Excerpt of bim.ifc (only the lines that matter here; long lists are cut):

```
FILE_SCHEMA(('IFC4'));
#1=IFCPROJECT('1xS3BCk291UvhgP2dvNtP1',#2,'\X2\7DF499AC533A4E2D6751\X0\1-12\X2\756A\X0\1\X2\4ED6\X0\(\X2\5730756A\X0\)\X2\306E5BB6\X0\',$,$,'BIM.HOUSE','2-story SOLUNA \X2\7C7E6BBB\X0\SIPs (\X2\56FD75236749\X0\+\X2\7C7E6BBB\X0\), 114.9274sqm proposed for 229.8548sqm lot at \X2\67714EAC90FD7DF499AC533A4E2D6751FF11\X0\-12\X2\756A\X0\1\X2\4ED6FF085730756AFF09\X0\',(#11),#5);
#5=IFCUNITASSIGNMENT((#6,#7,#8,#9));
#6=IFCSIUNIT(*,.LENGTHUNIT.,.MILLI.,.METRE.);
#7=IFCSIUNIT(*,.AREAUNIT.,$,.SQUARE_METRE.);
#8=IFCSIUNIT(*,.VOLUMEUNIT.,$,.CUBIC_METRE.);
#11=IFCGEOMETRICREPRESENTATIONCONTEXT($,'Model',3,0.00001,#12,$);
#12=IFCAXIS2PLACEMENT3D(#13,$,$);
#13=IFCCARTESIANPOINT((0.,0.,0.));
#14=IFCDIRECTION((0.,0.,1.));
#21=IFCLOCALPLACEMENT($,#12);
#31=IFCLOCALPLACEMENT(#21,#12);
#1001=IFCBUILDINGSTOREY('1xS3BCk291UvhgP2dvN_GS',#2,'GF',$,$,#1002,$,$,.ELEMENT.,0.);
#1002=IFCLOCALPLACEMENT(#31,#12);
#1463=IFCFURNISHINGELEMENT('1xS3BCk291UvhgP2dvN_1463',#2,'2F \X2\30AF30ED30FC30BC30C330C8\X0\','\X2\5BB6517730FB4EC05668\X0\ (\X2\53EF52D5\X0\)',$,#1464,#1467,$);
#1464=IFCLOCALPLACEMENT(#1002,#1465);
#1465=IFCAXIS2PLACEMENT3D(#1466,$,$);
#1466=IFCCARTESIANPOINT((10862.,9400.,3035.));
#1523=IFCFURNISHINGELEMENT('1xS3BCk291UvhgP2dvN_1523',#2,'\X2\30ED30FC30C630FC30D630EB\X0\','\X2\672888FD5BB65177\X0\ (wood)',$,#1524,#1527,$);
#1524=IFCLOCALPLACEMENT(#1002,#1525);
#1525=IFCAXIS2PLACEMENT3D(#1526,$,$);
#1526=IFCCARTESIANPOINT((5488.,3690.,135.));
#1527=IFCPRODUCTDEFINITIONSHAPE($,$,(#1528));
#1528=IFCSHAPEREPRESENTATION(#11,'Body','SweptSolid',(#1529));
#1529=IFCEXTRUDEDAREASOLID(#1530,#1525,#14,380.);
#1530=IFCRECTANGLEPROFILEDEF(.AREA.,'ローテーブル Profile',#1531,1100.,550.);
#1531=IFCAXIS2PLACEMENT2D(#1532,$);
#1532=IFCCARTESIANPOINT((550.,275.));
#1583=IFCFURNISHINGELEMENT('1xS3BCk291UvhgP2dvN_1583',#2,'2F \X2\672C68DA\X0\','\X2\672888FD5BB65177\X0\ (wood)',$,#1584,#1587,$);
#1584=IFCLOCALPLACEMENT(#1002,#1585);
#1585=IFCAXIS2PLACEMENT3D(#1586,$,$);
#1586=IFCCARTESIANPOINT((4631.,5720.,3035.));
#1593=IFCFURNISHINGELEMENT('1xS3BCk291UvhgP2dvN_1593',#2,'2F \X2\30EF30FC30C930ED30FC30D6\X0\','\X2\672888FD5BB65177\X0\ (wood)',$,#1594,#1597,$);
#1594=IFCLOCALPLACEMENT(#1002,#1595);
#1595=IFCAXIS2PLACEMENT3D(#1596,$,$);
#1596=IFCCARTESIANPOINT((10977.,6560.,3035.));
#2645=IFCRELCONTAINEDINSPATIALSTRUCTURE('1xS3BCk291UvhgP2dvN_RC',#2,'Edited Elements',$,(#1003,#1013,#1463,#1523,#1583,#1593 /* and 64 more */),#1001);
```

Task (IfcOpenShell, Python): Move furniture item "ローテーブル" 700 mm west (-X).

```python
import ifcopenshell
import ifcopenshell.api.geometry
import ifcopenshell.util.placement

model = ifcopenshell.open("bim.ifc")

item = model.by_guid("1xS3BCk291UvhgP2dvN_1523")
matrix = ifcopenshell.util.placement.get_local_placement(item.ObjectPlacement)
matrix[0, 3] -= 700.0
ifcopenshell.api.geometry.edit_object_placement(model, product=item, matrix=matrix, is_si=False)

print(ifcopenshell.util.placement.get_local_placement(item.ObjectPlacement).round(3) + 0.0)

model.write("bim_updated.ifc")
```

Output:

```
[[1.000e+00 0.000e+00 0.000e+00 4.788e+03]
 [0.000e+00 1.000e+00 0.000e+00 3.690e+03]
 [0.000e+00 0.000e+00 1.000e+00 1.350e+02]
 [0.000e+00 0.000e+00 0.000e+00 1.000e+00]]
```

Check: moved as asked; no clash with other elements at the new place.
